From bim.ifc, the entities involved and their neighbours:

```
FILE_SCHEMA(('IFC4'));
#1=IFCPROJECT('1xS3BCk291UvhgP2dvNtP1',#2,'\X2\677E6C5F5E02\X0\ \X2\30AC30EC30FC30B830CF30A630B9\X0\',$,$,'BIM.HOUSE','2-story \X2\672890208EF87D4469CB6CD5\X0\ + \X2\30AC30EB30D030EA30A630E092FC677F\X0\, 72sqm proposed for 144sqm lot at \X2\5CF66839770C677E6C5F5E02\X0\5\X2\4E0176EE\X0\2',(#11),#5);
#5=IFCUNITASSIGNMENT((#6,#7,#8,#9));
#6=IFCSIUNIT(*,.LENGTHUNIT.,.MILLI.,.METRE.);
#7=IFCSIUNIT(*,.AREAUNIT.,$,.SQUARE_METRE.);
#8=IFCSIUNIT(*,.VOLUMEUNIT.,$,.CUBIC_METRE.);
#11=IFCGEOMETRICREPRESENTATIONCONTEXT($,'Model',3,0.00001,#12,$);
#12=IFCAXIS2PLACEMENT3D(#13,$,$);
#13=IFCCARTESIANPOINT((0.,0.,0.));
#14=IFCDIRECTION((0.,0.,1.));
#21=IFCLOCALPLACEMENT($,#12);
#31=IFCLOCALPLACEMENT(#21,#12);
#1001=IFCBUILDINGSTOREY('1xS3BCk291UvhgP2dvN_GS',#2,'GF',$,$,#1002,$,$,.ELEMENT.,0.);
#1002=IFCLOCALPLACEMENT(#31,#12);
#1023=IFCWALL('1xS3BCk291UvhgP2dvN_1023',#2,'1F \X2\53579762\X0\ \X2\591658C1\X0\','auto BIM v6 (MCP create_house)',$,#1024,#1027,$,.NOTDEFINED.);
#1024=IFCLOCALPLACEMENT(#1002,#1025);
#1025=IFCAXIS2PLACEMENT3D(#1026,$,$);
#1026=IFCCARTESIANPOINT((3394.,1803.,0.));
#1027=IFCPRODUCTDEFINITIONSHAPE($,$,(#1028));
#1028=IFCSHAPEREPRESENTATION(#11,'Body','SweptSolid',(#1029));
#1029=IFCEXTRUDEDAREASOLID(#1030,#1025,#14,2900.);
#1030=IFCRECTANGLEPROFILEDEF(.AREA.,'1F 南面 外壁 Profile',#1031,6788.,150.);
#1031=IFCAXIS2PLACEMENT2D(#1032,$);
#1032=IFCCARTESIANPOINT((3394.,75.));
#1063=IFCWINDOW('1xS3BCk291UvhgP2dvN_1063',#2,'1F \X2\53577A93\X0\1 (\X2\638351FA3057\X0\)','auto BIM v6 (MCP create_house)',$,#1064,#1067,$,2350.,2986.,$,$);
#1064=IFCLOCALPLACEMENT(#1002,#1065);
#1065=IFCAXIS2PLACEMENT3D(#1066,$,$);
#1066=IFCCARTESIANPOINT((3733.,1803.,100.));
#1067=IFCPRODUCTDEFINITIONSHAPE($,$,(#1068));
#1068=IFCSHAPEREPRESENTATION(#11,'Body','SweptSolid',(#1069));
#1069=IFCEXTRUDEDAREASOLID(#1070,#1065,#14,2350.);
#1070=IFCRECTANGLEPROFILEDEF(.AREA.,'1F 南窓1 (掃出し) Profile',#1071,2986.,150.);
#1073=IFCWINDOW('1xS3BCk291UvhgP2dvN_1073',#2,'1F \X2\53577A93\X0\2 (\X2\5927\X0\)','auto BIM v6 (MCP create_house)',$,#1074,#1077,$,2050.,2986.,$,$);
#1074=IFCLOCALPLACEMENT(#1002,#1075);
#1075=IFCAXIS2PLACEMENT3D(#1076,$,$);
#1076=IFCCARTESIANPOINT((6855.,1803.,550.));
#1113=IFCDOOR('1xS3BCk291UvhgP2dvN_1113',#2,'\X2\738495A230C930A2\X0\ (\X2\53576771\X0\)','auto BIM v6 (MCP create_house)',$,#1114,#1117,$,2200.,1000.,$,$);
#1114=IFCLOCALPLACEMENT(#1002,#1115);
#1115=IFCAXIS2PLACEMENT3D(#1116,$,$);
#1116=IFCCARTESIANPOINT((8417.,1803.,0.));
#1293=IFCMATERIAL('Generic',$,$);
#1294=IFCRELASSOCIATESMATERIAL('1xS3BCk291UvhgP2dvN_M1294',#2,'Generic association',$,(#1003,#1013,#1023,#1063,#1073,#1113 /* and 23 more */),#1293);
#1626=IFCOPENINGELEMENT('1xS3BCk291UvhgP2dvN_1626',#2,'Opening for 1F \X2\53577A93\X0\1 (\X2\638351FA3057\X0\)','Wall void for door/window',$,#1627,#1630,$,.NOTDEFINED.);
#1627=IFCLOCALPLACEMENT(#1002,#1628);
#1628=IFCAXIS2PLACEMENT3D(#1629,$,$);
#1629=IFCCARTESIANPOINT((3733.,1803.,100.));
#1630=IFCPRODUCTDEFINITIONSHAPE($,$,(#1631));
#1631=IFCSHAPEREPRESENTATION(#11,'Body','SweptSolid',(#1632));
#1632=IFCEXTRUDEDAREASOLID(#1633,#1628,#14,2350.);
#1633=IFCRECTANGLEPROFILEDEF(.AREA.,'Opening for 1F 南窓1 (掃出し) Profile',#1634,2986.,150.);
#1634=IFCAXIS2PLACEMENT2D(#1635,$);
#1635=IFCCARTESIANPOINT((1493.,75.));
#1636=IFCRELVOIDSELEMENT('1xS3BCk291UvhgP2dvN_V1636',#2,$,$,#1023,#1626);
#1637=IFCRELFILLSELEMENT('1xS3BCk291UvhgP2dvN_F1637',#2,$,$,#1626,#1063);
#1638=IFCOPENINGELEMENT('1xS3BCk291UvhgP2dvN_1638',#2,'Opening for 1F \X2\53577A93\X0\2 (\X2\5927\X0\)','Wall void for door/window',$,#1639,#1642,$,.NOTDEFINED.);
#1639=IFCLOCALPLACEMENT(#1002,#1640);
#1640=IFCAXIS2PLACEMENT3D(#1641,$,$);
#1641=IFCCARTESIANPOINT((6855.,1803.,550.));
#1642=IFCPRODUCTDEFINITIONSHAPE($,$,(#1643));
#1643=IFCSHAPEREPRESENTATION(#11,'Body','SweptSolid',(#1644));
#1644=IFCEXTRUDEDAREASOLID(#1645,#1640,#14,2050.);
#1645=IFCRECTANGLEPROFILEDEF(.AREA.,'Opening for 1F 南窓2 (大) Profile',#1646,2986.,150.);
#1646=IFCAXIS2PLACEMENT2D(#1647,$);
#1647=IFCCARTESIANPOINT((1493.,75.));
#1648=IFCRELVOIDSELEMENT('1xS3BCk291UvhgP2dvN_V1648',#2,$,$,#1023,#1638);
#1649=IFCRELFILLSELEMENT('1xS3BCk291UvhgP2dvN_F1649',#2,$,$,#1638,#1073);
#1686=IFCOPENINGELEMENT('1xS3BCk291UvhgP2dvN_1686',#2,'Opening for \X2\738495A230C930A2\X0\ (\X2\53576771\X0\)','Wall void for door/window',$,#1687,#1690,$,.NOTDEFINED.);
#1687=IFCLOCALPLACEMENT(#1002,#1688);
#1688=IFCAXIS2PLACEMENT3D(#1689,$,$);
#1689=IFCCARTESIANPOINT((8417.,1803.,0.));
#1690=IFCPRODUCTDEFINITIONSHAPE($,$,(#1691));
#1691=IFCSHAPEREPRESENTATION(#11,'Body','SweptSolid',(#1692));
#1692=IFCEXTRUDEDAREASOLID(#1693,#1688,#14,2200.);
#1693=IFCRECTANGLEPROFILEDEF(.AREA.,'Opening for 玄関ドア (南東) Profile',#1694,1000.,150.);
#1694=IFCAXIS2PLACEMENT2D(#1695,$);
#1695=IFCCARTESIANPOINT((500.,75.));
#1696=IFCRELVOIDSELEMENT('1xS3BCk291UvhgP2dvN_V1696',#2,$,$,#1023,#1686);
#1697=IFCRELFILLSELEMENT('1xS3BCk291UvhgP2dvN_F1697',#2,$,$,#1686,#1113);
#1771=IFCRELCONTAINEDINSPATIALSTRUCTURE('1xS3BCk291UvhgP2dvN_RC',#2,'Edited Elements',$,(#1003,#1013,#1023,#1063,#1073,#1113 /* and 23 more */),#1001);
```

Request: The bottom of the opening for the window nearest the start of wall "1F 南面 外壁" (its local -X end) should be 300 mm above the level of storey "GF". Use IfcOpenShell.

```python
import numpy as np
import ifcopenshell
import ifcopenshell.api.geometry
import ifcopenshell.geom
import ifcopenshell.util.element
import ifcopenshell.util.placement
import ifcopenshell.util.shape
import ifcopenshell.util.unit

model = ifcopenshell.open("bim.ifc")
unit_scale = ifcopenshell.util.unit.calculate_unit_scale(model)

window = model.by_guid("1xS3BCk291UvhgP2dvN_1063")
opening = window.FillsVoids[0].RelatingOpeningElement
storey = ifcopenshell.util.element.get_container(window, ifc_class="IfcBuildingStorey")
level = ifcopenshell.util.placement.get_local_placement(storey.ObjectPlacement)[2, 3]

# The opening's origin need not be at the sill, so measure its lowest point.
shape = ifcopenshell.geom.create_shape(ifcopenshell.geom.settings(), opening)
bottom = ifcopenshell.util.shape.get_shape_bottom_elevation(shape, shape.geometry) / unit_scale
dz = level + 0.3 / unit_scale - bottom

shift = np.array([0.0, 0.0, dz])
# The window is not placed relative to its opening, so move both.
for product in (opening, window):
    matrix = ifcopenshell.util.placement.get_local_placement(product.ObjectPlacement)
    matrix[:3, 3] += shift
    ifcopenshell.api.geometry.edit_object_placement(model, product=product, matrix=matrix, is_si=False)

print(f"moved by {dz * unit_scale:+.3f} m")

model.write("bim-out.ifc")
```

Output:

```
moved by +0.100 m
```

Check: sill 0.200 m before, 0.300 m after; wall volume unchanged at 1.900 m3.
